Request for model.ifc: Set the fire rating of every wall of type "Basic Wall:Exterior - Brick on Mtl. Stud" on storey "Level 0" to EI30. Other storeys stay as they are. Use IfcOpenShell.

First a look at what the model holds.

```python
import ifcopenshell
import ifcopenshell.util.element

model = ifcopenshell.open("model.ifc")
print(model.schema)
storey = next(s for s in model.by_type("IfcBuildingStorey") if s.Name == "Level 0")
walls = [e for e in ifcopenshell.util.element.get_decomposition(storey) if e.is_a("IfcWall")]
seen = {}
for e in walls:
    element_type = ifcopenshell.util.element.get_type(e)
    key = (element_type.Name if element_type != e and element_type else None, ifcopenshell.util.element.get_pset(e, "Pset_WallCommon", "FireRating"))
    seen[key] = seen.get(key, 0) + 1
for (name, value), count in sorted(seen.items(), key=str):
    print(count, "x", name, "|", value)
```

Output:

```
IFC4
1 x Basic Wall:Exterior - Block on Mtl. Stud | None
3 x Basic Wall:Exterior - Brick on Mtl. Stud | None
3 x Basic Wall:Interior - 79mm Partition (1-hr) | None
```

```python
import ifcopenshell
import ifcopenshell.api.pset
import ifcopenshell.util.element

model = ifcopenshell.open("model.ifc")

storey = next(s for s in model.by_type("IfcBuildingStorey") if s.Name == "Level 0")
walls = [e for e in ifcopenshell.util.element.get_decomposition(storey) if e.is_a("IfcWall")]

count = 0
for e in walls:
    element_type = ifcopenshell.util.element.get_type(e)
    if element_type in (None, e) or element_type.Name != "Basic Wall:Exterior - Brick on Mtl. Stud":
        continue
    # add_pset returns the element's existing set when there is one.
    pset = ifcopenshell.api.pset.add_pset(model, product=e, name="Pset_WallCommon")
    ifcopenshell.api.pset.edit_pset(model, pset=pset, properties={"FireRating": "EI30"})
    count += 1

print(count, "walls updated")

model.write("model_edited.ifc")
```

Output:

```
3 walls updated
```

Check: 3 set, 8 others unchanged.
